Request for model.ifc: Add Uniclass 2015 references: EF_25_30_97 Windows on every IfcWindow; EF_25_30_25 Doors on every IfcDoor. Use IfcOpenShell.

First a look at what the model holds.

```python
import ifcopenshell

model = ifcopenshell.open("model.ifc")
print(model.schema)
print("classifications:", [c.Name for c in model.by_type("IfcClassification")])
for ifc_class in ("IfcDoor", "IfcRoof", "IfcStair", "IfcWall", "IfcWindow"):
    print(ifc_class, len(model.by_type(ifc_class)))
```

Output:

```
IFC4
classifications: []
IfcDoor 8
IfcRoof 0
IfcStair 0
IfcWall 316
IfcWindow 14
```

```python
import ifcopenshell
import ifcopenshell.api.classification

model = ifcopenshell.open("model.ifc")

system = ifcopenshell.api.classification.add_classification(model, classification="Uniclass 2015")

codes = {
    "IfcWindow": ("EF_25_30_97", "Windows"),
    "IfcDoor": ("EF_25_30_25", "Doors"),
}
for ifc_class, (code, name) in codes.items():
    products = model.by_type(ifc_class)
    ifcopenshell.api.classification.add_reference(
        model, products=products, classification=system, identification=code, name=name
    )
    print(code, len(products))

model.write("model_rev.ifc")
```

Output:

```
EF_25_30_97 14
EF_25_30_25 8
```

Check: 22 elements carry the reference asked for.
